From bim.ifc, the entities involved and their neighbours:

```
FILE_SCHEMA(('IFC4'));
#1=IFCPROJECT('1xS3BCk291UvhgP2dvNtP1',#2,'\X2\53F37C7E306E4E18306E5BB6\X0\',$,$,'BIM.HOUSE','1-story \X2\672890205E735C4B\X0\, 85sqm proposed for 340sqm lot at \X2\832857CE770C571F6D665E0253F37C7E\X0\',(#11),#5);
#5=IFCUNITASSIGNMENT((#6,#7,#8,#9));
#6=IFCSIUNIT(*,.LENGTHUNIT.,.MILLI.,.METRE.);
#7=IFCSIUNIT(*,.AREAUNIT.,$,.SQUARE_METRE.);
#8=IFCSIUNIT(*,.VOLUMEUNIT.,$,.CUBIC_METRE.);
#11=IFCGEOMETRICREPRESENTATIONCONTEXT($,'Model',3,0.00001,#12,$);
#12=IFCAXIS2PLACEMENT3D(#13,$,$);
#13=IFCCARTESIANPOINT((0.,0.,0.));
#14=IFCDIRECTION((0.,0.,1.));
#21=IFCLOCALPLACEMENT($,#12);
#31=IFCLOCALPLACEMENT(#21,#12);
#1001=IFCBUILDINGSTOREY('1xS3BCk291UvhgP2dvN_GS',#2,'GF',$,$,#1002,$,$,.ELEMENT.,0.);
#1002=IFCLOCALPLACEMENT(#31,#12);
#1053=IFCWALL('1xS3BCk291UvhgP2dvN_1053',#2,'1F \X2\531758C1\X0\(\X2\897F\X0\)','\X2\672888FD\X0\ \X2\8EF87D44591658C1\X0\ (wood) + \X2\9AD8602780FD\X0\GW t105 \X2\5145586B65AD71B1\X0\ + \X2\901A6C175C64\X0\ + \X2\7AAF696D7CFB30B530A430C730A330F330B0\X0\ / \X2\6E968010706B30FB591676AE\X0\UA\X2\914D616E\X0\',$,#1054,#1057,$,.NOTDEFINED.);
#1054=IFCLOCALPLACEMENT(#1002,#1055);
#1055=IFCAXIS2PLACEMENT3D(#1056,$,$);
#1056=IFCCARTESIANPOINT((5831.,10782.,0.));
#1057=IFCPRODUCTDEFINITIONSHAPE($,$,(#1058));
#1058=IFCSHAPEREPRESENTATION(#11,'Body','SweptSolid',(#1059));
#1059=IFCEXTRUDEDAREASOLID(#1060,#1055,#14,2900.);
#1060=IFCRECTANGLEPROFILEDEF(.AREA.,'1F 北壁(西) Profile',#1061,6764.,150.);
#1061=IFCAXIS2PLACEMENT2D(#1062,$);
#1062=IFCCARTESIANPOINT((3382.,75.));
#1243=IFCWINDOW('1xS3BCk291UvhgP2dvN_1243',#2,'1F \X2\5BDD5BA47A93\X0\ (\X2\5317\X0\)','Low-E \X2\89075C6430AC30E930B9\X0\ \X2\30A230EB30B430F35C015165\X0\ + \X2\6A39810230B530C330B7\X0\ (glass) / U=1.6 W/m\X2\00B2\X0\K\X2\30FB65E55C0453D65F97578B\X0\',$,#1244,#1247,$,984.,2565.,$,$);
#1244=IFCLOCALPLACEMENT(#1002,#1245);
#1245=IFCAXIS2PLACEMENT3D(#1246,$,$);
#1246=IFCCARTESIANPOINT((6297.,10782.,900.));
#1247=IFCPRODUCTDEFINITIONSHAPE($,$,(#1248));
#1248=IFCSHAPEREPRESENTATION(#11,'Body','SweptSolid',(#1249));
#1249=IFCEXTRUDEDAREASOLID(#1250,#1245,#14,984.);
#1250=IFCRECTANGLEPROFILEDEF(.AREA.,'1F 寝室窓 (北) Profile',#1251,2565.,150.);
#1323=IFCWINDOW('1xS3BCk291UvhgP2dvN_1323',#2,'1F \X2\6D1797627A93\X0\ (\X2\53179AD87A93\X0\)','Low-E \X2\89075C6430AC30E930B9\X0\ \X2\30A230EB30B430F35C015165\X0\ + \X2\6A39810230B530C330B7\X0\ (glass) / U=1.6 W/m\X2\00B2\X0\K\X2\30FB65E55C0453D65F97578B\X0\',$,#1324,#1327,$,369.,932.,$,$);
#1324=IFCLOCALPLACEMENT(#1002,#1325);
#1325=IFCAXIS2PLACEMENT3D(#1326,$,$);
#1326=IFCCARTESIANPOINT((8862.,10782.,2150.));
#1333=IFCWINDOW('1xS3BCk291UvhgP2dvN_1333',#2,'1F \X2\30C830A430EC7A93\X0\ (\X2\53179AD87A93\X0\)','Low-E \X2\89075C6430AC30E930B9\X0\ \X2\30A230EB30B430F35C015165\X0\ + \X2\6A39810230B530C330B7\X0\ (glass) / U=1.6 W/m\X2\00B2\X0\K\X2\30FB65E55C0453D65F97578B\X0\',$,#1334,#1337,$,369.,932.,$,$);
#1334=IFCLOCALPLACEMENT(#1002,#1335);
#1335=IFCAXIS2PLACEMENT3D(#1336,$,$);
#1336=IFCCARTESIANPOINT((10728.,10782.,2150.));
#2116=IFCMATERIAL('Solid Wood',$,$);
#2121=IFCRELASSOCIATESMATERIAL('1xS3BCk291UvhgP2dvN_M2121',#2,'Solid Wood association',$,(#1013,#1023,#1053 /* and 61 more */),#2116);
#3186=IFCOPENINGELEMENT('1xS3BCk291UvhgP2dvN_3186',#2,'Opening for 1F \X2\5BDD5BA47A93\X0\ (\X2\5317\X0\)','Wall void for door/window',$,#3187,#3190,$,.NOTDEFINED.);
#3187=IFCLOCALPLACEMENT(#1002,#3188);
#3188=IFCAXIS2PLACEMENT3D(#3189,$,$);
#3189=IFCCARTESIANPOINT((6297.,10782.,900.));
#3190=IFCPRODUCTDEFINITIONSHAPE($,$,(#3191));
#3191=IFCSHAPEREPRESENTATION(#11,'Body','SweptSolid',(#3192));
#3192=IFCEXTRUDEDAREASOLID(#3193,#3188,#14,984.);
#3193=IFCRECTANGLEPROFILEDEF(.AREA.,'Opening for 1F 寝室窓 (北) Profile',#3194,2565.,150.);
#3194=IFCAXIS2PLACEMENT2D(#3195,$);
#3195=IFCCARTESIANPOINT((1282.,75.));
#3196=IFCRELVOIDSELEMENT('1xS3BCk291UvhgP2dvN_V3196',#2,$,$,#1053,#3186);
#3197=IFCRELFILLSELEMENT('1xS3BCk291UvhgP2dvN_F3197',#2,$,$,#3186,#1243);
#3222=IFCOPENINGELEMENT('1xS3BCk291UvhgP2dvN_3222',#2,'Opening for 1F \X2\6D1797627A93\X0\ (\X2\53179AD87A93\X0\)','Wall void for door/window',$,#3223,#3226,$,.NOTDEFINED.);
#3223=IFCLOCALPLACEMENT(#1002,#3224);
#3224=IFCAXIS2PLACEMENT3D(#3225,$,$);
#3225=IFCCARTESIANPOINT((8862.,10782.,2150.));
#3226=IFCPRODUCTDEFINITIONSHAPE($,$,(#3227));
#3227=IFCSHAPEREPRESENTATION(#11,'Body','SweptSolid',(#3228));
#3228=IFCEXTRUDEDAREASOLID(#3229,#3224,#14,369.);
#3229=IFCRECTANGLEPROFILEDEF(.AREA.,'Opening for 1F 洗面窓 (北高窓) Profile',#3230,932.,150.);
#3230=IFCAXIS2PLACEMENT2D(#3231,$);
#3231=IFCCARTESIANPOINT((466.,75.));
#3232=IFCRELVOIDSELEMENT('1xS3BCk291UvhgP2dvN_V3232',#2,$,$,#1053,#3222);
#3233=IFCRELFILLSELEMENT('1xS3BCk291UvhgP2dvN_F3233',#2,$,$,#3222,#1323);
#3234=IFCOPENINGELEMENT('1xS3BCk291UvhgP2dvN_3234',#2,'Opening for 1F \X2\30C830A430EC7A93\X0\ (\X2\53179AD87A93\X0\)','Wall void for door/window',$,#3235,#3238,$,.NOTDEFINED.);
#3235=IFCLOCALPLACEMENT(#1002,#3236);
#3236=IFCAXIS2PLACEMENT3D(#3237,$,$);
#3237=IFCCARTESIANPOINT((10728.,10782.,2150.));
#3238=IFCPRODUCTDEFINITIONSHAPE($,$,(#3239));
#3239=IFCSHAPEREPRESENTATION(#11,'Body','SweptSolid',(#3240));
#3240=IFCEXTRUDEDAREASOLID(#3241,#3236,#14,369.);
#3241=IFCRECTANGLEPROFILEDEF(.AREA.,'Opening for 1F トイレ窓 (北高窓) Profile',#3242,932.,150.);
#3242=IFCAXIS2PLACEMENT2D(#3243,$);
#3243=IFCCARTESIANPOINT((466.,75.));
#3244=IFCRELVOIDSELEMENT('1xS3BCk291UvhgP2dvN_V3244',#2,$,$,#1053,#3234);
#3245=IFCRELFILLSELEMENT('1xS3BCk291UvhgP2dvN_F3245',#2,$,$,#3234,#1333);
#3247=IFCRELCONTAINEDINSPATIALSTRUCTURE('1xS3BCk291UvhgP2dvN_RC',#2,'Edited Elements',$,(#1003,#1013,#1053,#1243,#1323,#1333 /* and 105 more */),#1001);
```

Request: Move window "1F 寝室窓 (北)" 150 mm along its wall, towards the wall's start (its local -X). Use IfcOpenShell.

```python
import ifcopenshell
import ifcopenshell.api.geometry
import ifcopenshell.util.placement

model = ifcopenshell.open("bim.ifc")

window = model.by_guid("1xS3BCk291UvhgP2dvN_1243")
opening = window.FillsVoids[0].RelatingOpeningElement
wall = opening.VoidsElements[0].RelatingBuildingElement

wall_matrix = ifcopenshell.util.placement.get_local_placement(wall.ObjectPlacement)
shift = wall_matrix[:3, 0] * -150.0
before = ifcopenshell.util.placement.get_local_placement(window.ObjectPlacement)[:3, 3].copy()

# The window is not placed relative to its opening, so move both.
for product in (opening, window):
    matrix = ifcopenshell.util.placement.get_local_placement(product.ObjectPlacement)
    matrix[:3, 3] += shift
    ifcopenshell.api.geometry.edit_object_placement(model, product=product, matrix=matrix, is_si=False)

after = ifcopenshell.util.placement.get_local_placement(window.ObjectPlacement)[:3, 3]
print("window moved by", (after - before).round(3) + 0.0)

model.write("bim_rev.ifc")
```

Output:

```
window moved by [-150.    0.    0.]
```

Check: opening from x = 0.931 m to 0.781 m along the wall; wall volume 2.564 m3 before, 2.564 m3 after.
